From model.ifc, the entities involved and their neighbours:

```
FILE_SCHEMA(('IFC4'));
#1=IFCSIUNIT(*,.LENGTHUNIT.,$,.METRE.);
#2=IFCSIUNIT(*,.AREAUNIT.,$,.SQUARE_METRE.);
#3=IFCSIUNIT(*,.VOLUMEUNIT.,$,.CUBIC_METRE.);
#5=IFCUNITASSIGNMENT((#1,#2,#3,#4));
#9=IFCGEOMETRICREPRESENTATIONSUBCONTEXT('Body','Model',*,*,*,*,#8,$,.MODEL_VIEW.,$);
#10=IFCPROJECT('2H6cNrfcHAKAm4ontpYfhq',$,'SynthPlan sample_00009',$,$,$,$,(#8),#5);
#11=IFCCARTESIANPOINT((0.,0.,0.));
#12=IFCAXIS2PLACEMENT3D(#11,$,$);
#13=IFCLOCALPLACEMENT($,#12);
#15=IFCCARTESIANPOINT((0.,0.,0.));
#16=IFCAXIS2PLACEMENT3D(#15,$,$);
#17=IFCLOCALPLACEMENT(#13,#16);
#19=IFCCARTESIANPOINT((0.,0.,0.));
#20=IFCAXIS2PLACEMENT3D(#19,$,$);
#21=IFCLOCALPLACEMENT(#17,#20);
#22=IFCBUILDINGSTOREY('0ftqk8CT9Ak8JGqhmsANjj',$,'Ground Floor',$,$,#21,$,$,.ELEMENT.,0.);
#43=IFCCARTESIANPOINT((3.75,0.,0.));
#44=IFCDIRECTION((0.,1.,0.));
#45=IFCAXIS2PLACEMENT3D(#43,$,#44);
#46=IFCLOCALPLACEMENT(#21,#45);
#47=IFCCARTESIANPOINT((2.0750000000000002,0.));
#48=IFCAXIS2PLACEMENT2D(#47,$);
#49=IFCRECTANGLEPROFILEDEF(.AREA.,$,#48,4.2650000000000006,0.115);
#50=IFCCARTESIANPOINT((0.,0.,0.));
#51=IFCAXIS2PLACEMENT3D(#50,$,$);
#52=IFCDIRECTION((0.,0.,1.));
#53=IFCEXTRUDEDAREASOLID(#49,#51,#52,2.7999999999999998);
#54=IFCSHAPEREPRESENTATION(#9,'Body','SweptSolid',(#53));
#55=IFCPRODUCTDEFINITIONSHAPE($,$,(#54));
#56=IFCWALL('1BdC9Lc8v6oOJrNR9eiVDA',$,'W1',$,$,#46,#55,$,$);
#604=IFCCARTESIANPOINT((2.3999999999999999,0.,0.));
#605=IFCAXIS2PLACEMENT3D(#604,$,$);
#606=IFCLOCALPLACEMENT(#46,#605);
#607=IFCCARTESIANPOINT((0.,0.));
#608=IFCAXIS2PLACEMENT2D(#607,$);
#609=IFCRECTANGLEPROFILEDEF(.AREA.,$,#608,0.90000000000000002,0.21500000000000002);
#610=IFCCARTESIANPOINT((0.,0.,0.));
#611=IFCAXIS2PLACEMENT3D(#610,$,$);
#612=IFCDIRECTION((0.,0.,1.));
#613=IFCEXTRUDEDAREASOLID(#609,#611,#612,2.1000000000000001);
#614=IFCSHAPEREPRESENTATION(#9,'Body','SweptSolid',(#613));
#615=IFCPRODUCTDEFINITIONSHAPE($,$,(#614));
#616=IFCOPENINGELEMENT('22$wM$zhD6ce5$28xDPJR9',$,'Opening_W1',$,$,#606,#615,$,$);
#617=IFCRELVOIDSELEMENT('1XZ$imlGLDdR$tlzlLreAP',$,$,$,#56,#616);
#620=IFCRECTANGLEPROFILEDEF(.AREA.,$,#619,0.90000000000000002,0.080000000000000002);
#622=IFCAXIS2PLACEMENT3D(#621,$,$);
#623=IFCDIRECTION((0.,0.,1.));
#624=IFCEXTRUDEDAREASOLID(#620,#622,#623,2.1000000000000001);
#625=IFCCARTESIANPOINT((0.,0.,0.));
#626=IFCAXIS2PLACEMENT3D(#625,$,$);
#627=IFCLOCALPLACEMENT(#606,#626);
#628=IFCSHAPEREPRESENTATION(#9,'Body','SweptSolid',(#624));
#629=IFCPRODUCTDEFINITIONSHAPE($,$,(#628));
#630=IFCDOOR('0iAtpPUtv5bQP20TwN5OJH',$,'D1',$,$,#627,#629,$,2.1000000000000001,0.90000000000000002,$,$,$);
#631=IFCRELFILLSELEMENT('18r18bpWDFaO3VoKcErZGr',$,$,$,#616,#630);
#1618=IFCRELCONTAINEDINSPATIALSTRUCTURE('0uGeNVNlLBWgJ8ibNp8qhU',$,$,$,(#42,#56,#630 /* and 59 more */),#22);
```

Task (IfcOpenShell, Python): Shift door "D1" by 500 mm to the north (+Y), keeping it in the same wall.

```python
import ifcopenshell
import ifcopenshell.api.geometry
import ifcopenshell.util.placement

model = ifcopenshell.open("model.ifc")

door = model.by_guid("0iAtpPUtv5bQP20TwN5OJH")
opening = door.FillsVoids[0].RelatingOpeningElement
wall = opening.VoidsElements[0].RelatingBuildingElement

wall_matrix = ifcopenshell.util.placement.get_local_placement(wall.ObjectPlacement)
shift = wall_matrix[:3, 0] * 0.5
before = ifcopenshell.util.placement.get_local_placement(door.ObjectPlacement)[:3, 3].copy()

# The door is placed relative to its opening, so it follows when the opening moves.
matrix = ifcopenshell.util.placement.get_local_placement(opening.ObjectPlacement)
matrix[:3, 3] += shift
ifcopenshell.api.geometry.edit_object_placement(
    model, product=opening, matrix=matrix, is_si=False, should_transform_children=True
)

after = ifcopenshell.util.placement.get_local_placement(door.ObjectPlacement)[:3, 3]
print("door moved by", (after - before).round(3) + 0.0)

model.write("model_v2.ifc")
```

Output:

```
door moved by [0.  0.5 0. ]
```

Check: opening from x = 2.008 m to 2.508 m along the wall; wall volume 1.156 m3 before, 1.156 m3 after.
